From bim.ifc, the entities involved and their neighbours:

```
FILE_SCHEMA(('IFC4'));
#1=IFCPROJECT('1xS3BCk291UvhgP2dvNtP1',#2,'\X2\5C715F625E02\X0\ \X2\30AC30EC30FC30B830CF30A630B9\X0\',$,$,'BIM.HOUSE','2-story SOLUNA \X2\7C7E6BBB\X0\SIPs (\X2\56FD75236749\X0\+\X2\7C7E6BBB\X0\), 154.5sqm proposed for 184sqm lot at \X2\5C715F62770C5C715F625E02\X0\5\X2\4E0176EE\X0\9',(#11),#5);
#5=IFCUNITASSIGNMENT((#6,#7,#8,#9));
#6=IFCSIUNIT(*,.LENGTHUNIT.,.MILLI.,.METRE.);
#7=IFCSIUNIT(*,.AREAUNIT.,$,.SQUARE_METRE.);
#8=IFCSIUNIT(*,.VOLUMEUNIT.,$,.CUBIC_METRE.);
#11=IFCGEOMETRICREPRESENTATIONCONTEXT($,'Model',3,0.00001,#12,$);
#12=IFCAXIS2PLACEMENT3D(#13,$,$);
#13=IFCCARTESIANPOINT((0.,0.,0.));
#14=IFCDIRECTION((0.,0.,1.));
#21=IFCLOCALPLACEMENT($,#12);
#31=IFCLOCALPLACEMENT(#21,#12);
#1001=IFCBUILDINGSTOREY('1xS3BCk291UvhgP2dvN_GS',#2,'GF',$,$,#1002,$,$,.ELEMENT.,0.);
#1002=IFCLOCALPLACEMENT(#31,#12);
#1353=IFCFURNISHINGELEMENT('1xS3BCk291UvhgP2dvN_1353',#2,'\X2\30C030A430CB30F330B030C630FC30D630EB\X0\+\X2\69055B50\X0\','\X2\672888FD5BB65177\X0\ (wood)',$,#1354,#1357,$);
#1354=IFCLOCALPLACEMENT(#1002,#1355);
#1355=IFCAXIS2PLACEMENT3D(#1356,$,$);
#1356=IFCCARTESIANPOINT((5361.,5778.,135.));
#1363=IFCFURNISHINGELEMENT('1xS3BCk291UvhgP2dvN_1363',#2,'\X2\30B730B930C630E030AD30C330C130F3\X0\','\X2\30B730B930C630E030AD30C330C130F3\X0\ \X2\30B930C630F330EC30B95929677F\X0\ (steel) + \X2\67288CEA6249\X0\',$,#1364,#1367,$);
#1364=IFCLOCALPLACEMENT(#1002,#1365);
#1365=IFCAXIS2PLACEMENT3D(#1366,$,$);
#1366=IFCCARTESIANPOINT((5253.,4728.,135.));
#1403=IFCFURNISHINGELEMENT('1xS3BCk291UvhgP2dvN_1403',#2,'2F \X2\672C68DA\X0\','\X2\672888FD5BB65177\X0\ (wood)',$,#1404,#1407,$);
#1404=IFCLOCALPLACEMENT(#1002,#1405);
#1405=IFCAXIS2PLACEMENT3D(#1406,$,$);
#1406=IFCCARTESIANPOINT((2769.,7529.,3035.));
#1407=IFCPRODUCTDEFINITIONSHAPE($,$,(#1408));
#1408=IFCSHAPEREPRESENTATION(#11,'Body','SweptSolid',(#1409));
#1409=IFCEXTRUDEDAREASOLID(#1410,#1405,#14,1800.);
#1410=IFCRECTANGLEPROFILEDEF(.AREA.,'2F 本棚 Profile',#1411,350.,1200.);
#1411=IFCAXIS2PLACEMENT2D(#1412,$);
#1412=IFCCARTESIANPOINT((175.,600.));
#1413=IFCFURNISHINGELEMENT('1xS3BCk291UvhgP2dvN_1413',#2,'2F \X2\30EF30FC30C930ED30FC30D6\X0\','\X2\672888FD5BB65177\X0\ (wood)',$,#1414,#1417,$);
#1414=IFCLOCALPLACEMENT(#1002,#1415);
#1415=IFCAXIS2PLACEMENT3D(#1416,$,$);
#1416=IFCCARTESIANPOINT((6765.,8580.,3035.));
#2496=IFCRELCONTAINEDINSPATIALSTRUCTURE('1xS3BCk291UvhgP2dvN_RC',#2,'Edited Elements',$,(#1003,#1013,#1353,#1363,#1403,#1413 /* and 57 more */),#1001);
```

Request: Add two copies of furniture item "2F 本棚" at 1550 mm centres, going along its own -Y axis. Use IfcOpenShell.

```python
import ifcopenshell
import ifcopenshell.api.geometry
import ifcopenshell.api.root
import ifcopenshell.util.element
import ifcopenshell.util.placement

model = ifcopenshell.open("bim.ifc")


def reuse_history(source, copy):
    """copy_class also copies each property set's owner history, people and application; keep the originals."""
    for rel in copy.IsDefinedBy:
        if rel.is_a("IfcRelDefinesByProperties") and (history := rel.RelatingPropertyDefinition.OwnerHistory):
            rel.RelatingPropertyDefinition.OwnerHistory = source.OwnerHistory
            ifcopenshell.util.element.remove_deep2(model, history)


source = model.by_id(1403)
base = ifcopenshell.util.placement.get_local_placement(source.ObjectPlacement)
step = -base[:3, 1] * 1550.0

for i in range(1, 3):
    copy = ifcopenshell.api.root.copy_class(model, product=source)
    copy.Representation = ifcopenshell.util.element.copy_deep(
        model, source.Representation, exclude=["IfcGeometricRepresentationContext", "IfcRepresentationMap"]
    )
    reuse_history(source, copy)
    matrix = base.copy()
    matrix[:3, 3] += i * step
    print("added at", matrix[:3, 3].round(3) + 0.0)
    ifcopenshell.api.geometry.edit_object_placement(model, product=copy, matrix=matrix, is_si=False)

model.write("bim_edited.ifc")
```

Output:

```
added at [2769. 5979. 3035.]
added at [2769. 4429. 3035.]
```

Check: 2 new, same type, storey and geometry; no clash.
